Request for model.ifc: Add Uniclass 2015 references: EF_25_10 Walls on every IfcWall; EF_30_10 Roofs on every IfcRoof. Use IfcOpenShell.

First a look at what the model holds.

```python
import ifcopenshell

model = ifcopenshell.open("model.ifc")
print(model.schema)
print("classifications:", [c.Name for c in model.by_type("IfcClassification")])
for ifc_class in ("IfcDoor", "IfcRoof", "IfcStair", "IfcWall", "IfcWindow"):
    print(ifc_class, len(model.by_type(ifc_class)))
```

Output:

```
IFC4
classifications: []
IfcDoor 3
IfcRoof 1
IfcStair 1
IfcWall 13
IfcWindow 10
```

```python
import ifcopenshell
import ifcopenshell.api.classification

model = ifcopenshell.open("model.ifc")

system = ifcopenshell.api.classification.add_classification(model, classification="Uniclass 2015")

codes = {
    "IfcWall": ("EF_25_10", "Walls"),
    "IfcRoof": ("EF_30_10", "Roofs"),
}
for ifc_class, (code, name) in codes.items():
    products = model.by_type(ifc_class)
    ifcopenshell.api.classification.add_reference(
        model, products=products, classification=system, identification=code, name=name
    )
    print(code, len(products))

model.write("model_edited.ifc")
```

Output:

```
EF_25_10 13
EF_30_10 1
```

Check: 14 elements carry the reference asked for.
